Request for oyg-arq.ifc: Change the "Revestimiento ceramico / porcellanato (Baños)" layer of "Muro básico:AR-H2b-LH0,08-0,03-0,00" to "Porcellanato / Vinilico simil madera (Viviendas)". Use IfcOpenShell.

First a look at what the model holds.

```python
import ifcopenshell
import ifcopenshell.util.element

model = ifcopenshell.open("oyg-arq.ifc")
print(model.schema)
for layer_set in model.by_type("IfcMaterialLayerSet"):
    if layer_set.LayerSetName == "Muro básico:AR-H2b-LH0,08-0,03-0,00":
        for layer in layer_set.MaterialLayers:
            print(layer.id(), layer.Material and layer.Material.Name, layer.LayerThickness, sep=" | ")
        print(len(ifcopenshell.util.element.get_elements_by_material(model, layer_set)), "elements and types use it")
print(sorted(m.Name for m in model.by_type("IfcMaterial") if m.Name)[:60])
```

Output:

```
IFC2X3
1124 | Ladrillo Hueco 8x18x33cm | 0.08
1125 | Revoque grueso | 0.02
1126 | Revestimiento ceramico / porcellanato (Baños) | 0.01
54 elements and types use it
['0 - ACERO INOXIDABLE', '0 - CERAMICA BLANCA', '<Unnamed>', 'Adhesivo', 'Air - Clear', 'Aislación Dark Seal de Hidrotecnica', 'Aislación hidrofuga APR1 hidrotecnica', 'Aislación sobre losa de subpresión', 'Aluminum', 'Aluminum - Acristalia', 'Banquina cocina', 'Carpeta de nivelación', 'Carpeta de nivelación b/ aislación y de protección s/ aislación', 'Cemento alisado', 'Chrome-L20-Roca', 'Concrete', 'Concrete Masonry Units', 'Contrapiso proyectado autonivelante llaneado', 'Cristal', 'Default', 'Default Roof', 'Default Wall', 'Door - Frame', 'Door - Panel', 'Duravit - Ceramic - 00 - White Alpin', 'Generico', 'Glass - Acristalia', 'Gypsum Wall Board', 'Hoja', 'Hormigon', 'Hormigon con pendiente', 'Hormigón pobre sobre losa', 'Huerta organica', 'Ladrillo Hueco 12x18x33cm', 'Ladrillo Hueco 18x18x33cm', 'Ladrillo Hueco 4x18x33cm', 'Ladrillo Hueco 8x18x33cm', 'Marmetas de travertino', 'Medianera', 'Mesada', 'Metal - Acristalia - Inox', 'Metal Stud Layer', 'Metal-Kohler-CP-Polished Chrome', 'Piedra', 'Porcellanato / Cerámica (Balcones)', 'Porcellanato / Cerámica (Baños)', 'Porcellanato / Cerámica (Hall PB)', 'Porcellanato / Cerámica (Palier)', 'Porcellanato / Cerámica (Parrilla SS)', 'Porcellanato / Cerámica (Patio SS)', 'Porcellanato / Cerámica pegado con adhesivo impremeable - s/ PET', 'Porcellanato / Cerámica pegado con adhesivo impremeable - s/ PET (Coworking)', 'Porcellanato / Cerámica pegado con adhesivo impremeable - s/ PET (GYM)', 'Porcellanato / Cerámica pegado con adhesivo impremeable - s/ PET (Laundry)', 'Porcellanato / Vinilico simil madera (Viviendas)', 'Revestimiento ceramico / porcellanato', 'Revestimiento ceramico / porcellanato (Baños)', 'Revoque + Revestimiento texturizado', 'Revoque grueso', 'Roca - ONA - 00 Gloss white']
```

```python
import ifcopenshell
import ifcopenshell.api.material

model = ifcopenshell.open("oyg-arq.ifc")

layer_set = next(s for s in model.by_type("IfcMaterialLayerSet") if s.LayerSetName == "Muro básico:AR-H2b-LH0,08-0,03-0,00")
layer = next(l for l in layer_set.MaterialLayers if l.Material and l.Material.Name == "Revestimiento ceramico / porcellanato (Baños)")
material = next(m for m in model.by_type("IfcMaterial") if m.Name == "Porcellanato / Vinilico simil madera (Viviendas)")

# Point this one layer at the other material; renaming the old one would change it everywhere.
ifcopenshell.api.material.edit_layer(model, layer=layer, attributes={}, material=material)

print([l.Material.Name if l.Material else None for l in layer_set.MaterialLayers])

model.write("oyg-arq_rev.ifc")
```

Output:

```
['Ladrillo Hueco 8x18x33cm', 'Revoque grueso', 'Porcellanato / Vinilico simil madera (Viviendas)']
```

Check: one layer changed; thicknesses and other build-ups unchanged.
